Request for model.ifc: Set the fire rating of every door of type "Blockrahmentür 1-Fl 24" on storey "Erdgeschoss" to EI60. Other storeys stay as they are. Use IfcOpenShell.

First a look at what the model holds.

```python
import ifcopenshell
import ifcopenshell.util.element

model = ifcopenshell.open("model.ifc")
print(model.schema)
storey = next(s for s in model.by_type("IfcBuildingStorey") if s.Name == "Erdgeschoss")
doors = [e for e in ifcopenshell.util.element.get_decomposition(storey) if e.is_a("IfcDoor")]
seen = {}
for e in doors:
    element_type = ifcopenshell.util.element.get_type(e)
    key = (element_type.Name if element_type != e and element_type else None, ifcopenshell.util.element.get_pset(e, "Pset_DoorCommon", "FireRating"))
    seen[key] = seen.get(key, 0) + 1
for (name, value), count in sorted(seen.items(), key=str):
    print(count, "x", name, "|", value)
```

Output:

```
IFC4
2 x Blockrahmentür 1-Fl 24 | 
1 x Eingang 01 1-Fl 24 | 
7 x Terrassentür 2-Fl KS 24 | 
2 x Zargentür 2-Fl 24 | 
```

```python
import ifcopenshell
import ifcopenshell.api.pset
import ifcopenshell.util.element

model = ifcopenshell.open("model.ifc")

storey = next(s for s in model.by_type("IfcBuildingStorey") if s.Name == "Erdgeschoss")
doors = [e for e in ifcopenshell.util.element.get_decomposition(storey) if e.is_a("IfcDoor")]

count = 0
for e in doors:
    element_type = ifcopenshell.util.element.get_type(e)
    if element_type in (None, e) or element_type.Name != "Blockrahmentür 1-Fl 24":
        continue
    # add_pset returns the element's existing set when there is one.
    pset = ifcopenshell.api.pset.add_pset(model, product=e, name="Pset_DoorCommon")
    ifcopenshell.api.pset.edit_pset(model, pset=pset, properties={"FireRating": "EI60"})
    count += 1

print(count, "doors updated")

model.write("model-out.ifc")
```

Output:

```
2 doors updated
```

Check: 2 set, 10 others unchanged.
